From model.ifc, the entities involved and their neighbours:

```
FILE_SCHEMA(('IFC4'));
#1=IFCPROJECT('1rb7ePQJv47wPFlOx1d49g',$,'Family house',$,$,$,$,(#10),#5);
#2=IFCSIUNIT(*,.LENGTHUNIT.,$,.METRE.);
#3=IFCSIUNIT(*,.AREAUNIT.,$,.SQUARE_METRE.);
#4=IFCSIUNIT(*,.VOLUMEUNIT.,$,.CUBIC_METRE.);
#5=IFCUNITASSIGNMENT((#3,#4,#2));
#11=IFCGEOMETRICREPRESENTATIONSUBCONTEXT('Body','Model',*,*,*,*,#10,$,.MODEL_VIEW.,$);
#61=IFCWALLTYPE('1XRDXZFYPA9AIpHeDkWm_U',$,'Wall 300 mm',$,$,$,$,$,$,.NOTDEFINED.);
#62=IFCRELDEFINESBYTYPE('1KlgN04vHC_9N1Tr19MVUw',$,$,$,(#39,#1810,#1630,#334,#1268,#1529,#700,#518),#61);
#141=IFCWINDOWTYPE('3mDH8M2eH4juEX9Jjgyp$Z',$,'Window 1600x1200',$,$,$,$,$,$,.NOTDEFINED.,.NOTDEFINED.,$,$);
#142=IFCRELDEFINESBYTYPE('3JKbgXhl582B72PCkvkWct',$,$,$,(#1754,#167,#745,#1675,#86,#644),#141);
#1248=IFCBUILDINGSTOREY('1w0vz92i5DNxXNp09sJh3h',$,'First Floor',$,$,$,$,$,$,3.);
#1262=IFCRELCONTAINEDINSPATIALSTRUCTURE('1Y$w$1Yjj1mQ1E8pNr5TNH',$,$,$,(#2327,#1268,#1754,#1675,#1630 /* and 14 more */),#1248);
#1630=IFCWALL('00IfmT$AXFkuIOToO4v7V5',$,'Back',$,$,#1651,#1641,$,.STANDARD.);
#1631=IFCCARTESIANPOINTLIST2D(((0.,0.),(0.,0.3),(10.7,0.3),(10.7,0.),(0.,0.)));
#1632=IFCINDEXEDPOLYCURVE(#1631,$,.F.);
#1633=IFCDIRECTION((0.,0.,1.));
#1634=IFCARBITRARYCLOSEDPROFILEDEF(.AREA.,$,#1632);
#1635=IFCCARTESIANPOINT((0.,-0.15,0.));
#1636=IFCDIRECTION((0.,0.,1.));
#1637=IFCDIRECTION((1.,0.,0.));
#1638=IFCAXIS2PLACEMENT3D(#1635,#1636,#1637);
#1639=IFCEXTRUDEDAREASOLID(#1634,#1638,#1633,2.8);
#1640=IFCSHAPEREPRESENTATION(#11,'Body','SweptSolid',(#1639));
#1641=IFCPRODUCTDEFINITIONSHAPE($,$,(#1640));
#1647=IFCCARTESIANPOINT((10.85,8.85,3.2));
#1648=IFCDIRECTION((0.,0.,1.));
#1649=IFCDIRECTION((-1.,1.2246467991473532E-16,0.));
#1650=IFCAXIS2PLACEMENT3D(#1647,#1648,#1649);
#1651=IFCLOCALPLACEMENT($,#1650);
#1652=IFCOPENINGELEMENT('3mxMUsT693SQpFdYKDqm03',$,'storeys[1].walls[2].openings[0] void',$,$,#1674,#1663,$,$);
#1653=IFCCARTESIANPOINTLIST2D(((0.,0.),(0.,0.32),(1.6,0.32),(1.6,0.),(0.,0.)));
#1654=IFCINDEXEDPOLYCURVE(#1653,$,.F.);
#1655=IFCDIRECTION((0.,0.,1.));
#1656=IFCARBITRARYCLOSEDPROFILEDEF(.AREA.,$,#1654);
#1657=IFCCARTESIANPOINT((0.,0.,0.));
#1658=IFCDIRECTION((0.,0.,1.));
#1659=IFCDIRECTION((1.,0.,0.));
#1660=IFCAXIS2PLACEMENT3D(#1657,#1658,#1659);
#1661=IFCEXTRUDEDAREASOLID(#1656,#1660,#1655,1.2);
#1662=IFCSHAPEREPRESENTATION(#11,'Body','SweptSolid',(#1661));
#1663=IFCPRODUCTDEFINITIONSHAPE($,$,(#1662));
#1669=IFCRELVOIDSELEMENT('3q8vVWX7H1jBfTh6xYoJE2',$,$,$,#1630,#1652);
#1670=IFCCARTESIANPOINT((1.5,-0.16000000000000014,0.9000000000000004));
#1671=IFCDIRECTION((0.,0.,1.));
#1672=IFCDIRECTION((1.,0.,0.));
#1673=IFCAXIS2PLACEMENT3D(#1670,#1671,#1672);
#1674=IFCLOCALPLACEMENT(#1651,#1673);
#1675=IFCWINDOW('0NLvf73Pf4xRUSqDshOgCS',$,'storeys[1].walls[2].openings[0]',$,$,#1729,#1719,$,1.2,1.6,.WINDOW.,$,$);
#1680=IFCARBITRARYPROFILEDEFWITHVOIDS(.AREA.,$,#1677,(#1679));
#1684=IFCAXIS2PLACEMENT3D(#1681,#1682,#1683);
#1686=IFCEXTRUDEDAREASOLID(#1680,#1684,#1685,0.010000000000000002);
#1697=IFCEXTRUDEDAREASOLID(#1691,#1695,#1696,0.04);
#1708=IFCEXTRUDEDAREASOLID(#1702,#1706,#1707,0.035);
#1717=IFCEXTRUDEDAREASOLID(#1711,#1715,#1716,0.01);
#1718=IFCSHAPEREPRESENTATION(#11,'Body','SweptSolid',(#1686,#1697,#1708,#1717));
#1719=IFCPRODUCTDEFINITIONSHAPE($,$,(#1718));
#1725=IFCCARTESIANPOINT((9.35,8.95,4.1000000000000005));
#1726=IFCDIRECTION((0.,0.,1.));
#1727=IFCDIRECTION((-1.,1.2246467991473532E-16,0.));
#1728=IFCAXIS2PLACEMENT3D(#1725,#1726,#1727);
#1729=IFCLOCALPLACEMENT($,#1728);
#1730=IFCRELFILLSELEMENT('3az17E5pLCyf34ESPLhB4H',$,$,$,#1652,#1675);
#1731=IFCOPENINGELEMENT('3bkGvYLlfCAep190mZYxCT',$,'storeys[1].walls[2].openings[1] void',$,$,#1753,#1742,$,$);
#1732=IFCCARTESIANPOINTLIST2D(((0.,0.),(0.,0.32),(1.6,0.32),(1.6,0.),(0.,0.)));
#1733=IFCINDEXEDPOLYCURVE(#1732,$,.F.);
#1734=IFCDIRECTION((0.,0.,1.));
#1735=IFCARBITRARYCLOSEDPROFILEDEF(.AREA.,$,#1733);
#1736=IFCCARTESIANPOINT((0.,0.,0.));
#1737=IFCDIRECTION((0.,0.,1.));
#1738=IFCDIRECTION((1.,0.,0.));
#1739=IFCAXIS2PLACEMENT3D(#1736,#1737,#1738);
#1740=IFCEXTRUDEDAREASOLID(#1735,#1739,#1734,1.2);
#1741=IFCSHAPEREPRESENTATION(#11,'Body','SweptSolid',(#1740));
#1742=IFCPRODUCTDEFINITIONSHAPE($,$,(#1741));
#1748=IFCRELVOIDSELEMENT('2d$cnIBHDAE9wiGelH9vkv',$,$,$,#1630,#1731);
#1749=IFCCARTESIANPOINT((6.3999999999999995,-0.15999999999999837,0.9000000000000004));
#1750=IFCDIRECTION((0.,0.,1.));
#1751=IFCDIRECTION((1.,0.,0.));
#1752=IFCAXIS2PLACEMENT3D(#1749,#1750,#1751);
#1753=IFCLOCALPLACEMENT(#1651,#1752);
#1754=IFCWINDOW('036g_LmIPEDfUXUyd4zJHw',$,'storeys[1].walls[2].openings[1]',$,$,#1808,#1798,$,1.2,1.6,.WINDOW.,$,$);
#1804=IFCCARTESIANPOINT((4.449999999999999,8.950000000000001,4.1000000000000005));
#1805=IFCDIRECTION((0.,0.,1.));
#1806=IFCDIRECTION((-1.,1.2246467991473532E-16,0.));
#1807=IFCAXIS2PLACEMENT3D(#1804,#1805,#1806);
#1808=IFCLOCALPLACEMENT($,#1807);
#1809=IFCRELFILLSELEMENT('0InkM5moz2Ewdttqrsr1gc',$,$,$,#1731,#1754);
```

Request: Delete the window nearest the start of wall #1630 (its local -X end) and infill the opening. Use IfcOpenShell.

```python
import ifcopenshell
import ifcopenshell.api.feature
import ifcopenshell.api.root
import ifcopenshell.geom
import ifcopenshell.util.shape

model = ifcopenshell.open("model.ifc")
settings = ifcopenshell.geom.settings()


def volume(element):
    """Net volume in cubic metres, openings subtracted."""
    shape = ifcopenshell.geom.create_shape(settings, element)
    return ifcopenshell.util.shape.get_volume(shape.geometry)


window = model.by_id(1675)
opening = window.FillsVoids[0].RelatingOpeningElement
wall = opening.VoidsElements[0].RelatingBuildingElement
before = volume(wall)

ifcopenshell.api.root.remove_product(model, product=window)
ifcopenshell.api.feature.remove_feature(model, feature=opening)

after = volume(wall)

print(f"wall volume {before:.3f} -> {after:.3f} m3")

model.write("model_rev.ifc")
```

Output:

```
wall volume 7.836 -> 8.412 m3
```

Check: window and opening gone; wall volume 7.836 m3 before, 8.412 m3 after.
